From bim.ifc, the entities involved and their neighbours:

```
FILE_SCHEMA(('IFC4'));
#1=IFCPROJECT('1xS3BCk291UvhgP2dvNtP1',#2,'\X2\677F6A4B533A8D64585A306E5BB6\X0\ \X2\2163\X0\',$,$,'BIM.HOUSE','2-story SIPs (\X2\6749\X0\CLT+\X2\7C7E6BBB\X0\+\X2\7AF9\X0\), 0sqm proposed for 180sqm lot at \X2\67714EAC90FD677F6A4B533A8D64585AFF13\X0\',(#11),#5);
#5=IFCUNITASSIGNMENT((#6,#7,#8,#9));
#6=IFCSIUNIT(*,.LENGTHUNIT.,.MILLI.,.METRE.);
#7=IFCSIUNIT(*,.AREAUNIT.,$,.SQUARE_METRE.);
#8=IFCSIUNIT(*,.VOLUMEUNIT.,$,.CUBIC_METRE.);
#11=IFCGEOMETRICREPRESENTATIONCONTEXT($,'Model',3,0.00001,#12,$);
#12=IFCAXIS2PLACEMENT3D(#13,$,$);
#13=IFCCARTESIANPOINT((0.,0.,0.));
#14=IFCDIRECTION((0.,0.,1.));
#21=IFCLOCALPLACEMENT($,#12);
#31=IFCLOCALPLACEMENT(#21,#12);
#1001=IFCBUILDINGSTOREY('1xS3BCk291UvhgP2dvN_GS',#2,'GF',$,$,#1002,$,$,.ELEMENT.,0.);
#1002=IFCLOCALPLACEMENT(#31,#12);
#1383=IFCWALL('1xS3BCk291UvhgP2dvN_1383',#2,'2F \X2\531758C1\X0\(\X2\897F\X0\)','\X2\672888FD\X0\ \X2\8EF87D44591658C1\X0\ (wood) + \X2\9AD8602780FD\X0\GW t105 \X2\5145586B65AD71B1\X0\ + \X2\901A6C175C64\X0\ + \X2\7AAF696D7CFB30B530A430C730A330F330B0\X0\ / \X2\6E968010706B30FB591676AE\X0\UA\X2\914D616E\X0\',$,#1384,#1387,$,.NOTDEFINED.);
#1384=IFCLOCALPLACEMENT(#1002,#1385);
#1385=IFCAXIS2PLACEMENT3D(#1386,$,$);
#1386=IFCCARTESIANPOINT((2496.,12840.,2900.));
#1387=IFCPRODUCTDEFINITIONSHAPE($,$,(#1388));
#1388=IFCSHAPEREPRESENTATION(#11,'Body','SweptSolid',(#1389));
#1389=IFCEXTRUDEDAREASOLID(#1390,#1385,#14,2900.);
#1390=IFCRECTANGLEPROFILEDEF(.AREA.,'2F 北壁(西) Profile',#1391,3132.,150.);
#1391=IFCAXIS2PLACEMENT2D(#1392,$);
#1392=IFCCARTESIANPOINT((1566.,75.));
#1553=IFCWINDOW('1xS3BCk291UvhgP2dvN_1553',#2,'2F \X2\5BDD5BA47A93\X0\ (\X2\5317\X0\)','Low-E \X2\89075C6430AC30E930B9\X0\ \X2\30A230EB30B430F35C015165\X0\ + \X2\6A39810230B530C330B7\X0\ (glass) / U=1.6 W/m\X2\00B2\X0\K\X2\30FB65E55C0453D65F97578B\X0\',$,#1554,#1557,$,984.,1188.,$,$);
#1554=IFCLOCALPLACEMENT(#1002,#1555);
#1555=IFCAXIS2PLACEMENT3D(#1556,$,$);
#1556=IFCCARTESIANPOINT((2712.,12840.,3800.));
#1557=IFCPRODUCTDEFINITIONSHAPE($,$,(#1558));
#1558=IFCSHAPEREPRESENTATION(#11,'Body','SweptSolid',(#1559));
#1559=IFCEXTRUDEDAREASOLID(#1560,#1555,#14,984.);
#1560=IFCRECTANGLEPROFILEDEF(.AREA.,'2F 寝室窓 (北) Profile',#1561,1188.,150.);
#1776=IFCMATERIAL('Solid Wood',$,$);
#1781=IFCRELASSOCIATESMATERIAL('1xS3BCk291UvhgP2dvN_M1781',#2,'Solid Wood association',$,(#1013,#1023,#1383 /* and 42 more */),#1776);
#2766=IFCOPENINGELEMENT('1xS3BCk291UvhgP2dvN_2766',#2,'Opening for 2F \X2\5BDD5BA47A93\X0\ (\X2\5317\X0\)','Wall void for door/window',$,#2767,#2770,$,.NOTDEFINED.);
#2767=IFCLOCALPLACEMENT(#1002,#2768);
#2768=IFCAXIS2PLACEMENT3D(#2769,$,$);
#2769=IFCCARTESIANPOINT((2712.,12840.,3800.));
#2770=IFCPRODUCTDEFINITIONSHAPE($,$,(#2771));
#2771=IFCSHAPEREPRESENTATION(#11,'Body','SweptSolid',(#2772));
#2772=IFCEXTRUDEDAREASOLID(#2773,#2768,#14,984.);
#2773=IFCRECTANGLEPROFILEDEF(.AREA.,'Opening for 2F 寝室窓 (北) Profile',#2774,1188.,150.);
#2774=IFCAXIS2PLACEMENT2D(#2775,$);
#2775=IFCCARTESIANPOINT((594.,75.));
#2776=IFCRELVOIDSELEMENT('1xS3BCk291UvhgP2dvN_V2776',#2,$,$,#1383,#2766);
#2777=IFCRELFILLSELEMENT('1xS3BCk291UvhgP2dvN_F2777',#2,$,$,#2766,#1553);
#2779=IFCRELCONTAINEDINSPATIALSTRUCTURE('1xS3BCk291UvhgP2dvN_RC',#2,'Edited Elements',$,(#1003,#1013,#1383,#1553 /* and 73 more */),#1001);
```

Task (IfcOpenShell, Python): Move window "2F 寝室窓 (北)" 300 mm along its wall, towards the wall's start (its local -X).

```python
import ifcopenshell
import ifcopenshell.api.geometry
import ifcopenshell.util.placement
import ifcopenshell.util.unit

model = ifcopenshell.open("bim.ifc")
unit_scale = ifcopenshell.util.unit.calculate_unit_scale(model)

window = model.by_guid("1xS3BCk291UvhgP2dvN_1553")
opening = window.FillsVoids[0].RelatingOpeningElement
wall = opening.VoidsElements[0].RelatingBuildingElement

wall_matrix = ifcopenshell.util.placement.get_local_placement(wall.ObjectPlacement)
shift = wall_matrix[:3, 0] * -0.3 / unit_scale
before = ifcopenshell.util.placement.get_local_placement(window.ObjectPlacement)[:3, 3].copy()

# The window is not placed relative to its opening, so move both.
for product in (opening, window):
    matrix = ifcopenshell.util.placement.get_local_placement(product.ObjectPlacement)
    matrix[:3, 3] += shift
    ifcopenshell.api.geometry.edit_object_placement(model, product=product, matrix=matrix, is_si=False)

after = ifcopenshell.util.placement.get_local_placement(window.ObjectPlacement)[:3, 3]
print("window moved by", (after - before).round(3) + 0.0)

model.write("bim_updated.ifc")
```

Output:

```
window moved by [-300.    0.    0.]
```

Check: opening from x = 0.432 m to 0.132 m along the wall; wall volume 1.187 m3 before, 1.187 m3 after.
